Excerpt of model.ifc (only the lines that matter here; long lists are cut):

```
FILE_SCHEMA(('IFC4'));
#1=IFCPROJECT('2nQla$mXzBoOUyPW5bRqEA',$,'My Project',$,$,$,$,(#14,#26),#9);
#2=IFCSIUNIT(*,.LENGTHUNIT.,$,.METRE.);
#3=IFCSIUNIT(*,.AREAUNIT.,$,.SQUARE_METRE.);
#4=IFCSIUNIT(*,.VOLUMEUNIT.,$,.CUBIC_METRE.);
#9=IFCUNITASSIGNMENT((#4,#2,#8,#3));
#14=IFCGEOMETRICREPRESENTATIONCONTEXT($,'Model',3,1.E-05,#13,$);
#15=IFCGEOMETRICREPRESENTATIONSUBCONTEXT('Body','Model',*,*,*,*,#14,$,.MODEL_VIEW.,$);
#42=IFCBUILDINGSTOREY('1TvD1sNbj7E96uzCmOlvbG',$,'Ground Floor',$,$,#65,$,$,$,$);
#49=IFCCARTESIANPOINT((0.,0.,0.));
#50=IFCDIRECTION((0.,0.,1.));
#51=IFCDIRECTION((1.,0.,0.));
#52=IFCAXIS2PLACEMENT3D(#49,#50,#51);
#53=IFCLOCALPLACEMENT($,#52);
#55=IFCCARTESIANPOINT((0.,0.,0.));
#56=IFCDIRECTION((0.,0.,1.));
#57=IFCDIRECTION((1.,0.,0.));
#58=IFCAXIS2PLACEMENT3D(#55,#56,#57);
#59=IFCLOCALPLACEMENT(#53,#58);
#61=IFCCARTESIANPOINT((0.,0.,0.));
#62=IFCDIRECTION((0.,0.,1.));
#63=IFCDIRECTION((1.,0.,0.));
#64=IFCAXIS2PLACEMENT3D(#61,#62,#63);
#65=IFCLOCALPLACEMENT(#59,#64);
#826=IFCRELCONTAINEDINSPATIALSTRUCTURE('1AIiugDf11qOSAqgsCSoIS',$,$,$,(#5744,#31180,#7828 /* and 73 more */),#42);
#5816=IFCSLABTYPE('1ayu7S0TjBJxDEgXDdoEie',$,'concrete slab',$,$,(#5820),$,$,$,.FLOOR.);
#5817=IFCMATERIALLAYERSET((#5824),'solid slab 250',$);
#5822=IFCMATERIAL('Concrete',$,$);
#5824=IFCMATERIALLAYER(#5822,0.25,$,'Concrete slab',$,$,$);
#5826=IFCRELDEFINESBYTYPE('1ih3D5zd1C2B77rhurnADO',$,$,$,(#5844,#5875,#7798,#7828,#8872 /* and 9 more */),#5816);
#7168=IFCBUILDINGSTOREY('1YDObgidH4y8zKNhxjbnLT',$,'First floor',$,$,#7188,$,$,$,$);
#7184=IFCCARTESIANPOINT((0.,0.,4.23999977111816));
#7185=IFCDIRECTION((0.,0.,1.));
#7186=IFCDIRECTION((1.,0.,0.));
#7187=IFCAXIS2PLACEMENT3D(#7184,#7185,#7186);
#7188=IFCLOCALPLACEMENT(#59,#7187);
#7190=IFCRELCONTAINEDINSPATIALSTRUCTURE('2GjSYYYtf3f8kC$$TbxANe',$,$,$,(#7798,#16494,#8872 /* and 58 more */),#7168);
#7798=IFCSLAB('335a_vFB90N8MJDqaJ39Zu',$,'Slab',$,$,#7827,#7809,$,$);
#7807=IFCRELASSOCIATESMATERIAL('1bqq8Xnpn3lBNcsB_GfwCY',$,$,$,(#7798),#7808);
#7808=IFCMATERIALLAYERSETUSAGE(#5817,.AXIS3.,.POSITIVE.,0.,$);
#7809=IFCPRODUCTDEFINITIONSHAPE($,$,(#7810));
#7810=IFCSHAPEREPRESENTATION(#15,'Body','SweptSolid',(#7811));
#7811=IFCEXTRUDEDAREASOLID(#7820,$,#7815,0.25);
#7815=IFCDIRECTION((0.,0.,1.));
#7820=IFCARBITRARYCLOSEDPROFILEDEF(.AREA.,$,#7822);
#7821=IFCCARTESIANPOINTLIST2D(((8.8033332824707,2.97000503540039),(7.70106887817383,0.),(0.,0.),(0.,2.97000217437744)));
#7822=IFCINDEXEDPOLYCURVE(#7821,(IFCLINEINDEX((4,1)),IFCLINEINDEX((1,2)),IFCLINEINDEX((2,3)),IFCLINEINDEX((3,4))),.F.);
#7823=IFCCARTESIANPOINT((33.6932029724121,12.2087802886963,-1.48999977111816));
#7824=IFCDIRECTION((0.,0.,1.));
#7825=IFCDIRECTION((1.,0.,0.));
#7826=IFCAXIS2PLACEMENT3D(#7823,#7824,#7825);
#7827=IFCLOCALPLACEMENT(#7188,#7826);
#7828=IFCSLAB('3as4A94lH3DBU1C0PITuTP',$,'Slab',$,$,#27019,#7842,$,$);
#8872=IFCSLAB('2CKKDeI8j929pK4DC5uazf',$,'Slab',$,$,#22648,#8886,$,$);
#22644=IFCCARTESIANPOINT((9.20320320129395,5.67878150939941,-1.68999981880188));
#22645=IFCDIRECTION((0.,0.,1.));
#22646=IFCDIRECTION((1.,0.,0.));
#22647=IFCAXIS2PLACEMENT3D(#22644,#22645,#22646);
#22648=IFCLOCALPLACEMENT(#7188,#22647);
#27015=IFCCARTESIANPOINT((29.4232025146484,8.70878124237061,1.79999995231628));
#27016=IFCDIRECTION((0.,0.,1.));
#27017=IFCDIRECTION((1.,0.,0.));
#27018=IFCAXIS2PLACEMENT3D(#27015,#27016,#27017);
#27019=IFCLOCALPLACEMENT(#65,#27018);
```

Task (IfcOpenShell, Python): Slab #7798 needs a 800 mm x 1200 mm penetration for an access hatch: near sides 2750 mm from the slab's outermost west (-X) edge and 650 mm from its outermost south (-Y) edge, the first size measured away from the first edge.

```python
import numpy as np
import ifcopenshell
import ifcopenshell.api.feature
import ifcopenshell.api.geometry
import ifcopenshell.api.root
import ifcopenshell.geom
import ifcopenshell.util.placement
import ifcopenshell.util.representation
import ifcopenshell.util.shape
import ifcopenshell.util.unit

model = ifcopenshell.open("model.ifc")
unit_scale = ifcopenshell.util.unit.calculate_unit_scale(model)
settings = ifcopenshell.geom.settings()


def volume(element):
    """Net volume in cubic metres, openings subtracted."""
    shape = ifcopenshell.geom.create_shape(settings, element)
    return ifcopenshell.util.shape.get_volume(shape.geometry)


slab = model.by_id(7798)
before = volume(slab)

# Extent in the slab's own axes, in metres. The edges named are its -X and -Y sides.
slab_shape = ifcopenshell.geom.create_shape(settings, slab)
vertices = ifcopenshell.util.shape.get_vertices(slab_shape.geometry)
x_min, y_min, bottom = vertices.min(axis=0)
top = vertices[:, 2].max()

opening = ifcopenshell.api.root.create_entity(model, ifc_class="IfcOpeningElement", name="Access hatch opening", predefined_type="OPENING")
context = ifcopenshell.util.representation.get_context(model, "Model", "Body", "MODEL_VIEW")
width, depth = 0.8, 1.2
outline = [(0.0, 0.0), (width, 0.0), (width, depth), (0.0, depth), (0.0, 0.0)]
# Overshoot both faces by 50 mm so the cut is clean.
shape = ifcopenshell.api.geometry.add_slab_representation(
    model, context=context, depth=top - bottom + 0.1, polyline=outline
)
ifcopenshell.api.geometry.assign_representation(model, product=opening, representation=shape)

matrix = ifcopenshell.util.placement.get_local_placement(slab.ObjectPlacement)
matrix[:, 3] = matrix @ np.append(np.array([x_min + 2.75, y_min + 0.65, bottom - 0.05]) / unit_scale, 1.0)
ifcopenshell.api.geometry.edit_object_placement(model, product=opening, matrix=matrix, is_si=False)
ifcopenshell.api.feature.add_feature(model, feature=opening, element=slab)

after = volume(slab)

print(f"slab volume {before:.3f} -> {after:.3f} m3")

model.write("model_edited.ifc")
```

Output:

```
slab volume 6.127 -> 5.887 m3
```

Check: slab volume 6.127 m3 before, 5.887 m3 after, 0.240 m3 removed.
